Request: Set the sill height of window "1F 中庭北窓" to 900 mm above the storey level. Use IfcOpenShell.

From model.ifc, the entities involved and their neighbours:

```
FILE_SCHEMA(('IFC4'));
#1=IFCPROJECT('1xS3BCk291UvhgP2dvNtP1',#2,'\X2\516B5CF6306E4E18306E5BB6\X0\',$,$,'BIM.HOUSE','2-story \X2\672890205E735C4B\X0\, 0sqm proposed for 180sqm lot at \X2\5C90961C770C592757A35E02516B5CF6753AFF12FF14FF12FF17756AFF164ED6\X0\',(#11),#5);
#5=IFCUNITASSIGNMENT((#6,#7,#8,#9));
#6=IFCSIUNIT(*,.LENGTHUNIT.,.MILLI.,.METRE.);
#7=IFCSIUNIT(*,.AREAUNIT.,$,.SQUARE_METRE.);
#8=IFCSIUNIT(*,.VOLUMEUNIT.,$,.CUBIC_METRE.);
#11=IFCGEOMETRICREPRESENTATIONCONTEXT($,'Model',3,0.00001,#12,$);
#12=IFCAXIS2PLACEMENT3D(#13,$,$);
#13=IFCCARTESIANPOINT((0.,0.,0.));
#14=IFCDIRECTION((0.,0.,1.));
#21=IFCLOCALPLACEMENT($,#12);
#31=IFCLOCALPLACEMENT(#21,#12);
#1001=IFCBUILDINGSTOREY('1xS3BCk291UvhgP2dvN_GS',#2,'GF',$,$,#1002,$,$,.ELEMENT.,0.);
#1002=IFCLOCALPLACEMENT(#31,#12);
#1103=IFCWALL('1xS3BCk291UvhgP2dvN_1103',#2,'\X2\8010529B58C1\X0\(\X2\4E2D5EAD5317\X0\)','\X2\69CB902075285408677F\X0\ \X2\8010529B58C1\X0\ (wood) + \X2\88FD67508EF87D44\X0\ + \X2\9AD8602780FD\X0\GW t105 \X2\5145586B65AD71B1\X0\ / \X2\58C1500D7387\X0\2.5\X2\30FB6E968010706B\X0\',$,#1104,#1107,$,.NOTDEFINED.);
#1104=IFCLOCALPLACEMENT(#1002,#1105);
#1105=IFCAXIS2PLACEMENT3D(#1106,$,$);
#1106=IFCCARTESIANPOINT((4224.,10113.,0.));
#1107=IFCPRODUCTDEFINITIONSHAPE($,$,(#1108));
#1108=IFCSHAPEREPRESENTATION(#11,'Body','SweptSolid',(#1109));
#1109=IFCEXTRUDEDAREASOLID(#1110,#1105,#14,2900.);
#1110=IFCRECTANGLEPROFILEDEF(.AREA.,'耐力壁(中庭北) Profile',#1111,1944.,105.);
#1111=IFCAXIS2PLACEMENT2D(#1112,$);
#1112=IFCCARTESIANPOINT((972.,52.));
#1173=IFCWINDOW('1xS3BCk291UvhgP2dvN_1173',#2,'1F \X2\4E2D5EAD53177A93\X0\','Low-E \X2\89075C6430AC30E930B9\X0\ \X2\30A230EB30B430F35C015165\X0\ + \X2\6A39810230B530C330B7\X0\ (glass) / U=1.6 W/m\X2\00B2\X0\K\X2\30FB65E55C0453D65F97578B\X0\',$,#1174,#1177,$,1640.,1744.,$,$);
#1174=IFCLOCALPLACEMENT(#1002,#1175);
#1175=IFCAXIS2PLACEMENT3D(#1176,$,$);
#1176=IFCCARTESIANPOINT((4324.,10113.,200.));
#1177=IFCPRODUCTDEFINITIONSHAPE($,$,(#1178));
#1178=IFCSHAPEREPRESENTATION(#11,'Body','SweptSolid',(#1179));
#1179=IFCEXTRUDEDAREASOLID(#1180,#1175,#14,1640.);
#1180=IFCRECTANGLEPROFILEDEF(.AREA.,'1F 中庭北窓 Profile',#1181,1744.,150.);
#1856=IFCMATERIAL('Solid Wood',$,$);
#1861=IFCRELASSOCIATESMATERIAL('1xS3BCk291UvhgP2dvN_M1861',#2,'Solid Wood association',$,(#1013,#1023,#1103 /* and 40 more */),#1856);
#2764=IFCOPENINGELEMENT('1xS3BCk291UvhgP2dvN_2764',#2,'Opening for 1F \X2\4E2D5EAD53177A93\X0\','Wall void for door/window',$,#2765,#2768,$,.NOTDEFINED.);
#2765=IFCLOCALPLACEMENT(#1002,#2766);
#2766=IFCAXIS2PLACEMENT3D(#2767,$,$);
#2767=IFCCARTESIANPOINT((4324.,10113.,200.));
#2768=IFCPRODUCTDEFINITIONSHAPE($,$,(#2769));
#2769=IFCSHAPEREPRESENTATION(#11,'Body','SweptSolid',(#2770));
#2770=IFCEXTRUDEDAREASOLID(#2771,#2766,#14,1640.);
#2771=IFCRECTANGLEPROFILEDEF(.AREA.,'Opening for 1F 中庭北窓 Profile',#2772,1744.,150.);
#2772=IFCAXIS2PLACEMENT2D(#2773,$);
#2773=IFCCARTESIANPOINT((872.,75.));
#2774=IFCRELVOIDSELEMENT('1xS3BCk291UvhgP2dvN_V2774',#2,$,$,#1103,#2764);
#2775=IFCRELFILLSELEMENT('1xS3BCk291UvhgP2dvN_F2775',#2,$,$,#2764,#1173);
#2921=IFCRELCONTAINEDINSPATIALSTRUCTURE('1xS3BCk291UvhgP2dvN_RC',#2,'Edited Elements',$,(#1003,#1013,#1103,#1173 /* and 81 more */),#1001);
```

```python
import numpy as np
import ifcopenshell
import ifcopenshell.api.geometry
import ifcopenshell.geom
import ifcopenshell.util.element
import ifcopenshell.util.placement
import ifcopenshell.util.shape
import ifcopenshell.util.unit

model = ifcopenshell.open("model.ifc")
unit_scale = ifcopenshell.util.unit.calculate_unit_scale(model)

window = model.by_guid("1xS3BCk291UvhgP2dvN_1173")
opening = window.FillsVoids[0].RelatingOpeningElement
storey = ifcopenshell.util.element.get_container(window, ifc_class="IfcBuildingStorey")
level = ifcopenshell.util.placement.get_local_placement(storey.ObjectPlacement)[2, 3]

# The opening's origin need not be at the sill, so measure its lowest point.
shape = ifcopenshell.geom.create_shape(ifcopenshell.geom.settings(), opening)
bottom = ifcopenshell.util.shape.get_shape_bottom_elevation(shape, shape.geometry) / unit_scale
dz = level + 0.9 / unit_scale - bottom

shift = np.array([0.0, 0.0, dz])
# The window is not placed relative to its opening, so move both.
for product in (opening, window):
    matrix = ifcopenshell.util.placement.get_local_placement(product.ObjectPlacement)
    matrix[:3, 3] += shift
    ifcopenshell.api.geometry.edit_object_placement(model, product=product, matrix=matrix, is_si=False)

print(f"moved by {dz * unit_scale:+.3f} m")

model.write("model_rev.ifc")
```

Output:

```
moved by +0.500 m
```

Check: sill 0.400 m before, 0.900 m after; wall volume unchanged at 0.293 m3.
